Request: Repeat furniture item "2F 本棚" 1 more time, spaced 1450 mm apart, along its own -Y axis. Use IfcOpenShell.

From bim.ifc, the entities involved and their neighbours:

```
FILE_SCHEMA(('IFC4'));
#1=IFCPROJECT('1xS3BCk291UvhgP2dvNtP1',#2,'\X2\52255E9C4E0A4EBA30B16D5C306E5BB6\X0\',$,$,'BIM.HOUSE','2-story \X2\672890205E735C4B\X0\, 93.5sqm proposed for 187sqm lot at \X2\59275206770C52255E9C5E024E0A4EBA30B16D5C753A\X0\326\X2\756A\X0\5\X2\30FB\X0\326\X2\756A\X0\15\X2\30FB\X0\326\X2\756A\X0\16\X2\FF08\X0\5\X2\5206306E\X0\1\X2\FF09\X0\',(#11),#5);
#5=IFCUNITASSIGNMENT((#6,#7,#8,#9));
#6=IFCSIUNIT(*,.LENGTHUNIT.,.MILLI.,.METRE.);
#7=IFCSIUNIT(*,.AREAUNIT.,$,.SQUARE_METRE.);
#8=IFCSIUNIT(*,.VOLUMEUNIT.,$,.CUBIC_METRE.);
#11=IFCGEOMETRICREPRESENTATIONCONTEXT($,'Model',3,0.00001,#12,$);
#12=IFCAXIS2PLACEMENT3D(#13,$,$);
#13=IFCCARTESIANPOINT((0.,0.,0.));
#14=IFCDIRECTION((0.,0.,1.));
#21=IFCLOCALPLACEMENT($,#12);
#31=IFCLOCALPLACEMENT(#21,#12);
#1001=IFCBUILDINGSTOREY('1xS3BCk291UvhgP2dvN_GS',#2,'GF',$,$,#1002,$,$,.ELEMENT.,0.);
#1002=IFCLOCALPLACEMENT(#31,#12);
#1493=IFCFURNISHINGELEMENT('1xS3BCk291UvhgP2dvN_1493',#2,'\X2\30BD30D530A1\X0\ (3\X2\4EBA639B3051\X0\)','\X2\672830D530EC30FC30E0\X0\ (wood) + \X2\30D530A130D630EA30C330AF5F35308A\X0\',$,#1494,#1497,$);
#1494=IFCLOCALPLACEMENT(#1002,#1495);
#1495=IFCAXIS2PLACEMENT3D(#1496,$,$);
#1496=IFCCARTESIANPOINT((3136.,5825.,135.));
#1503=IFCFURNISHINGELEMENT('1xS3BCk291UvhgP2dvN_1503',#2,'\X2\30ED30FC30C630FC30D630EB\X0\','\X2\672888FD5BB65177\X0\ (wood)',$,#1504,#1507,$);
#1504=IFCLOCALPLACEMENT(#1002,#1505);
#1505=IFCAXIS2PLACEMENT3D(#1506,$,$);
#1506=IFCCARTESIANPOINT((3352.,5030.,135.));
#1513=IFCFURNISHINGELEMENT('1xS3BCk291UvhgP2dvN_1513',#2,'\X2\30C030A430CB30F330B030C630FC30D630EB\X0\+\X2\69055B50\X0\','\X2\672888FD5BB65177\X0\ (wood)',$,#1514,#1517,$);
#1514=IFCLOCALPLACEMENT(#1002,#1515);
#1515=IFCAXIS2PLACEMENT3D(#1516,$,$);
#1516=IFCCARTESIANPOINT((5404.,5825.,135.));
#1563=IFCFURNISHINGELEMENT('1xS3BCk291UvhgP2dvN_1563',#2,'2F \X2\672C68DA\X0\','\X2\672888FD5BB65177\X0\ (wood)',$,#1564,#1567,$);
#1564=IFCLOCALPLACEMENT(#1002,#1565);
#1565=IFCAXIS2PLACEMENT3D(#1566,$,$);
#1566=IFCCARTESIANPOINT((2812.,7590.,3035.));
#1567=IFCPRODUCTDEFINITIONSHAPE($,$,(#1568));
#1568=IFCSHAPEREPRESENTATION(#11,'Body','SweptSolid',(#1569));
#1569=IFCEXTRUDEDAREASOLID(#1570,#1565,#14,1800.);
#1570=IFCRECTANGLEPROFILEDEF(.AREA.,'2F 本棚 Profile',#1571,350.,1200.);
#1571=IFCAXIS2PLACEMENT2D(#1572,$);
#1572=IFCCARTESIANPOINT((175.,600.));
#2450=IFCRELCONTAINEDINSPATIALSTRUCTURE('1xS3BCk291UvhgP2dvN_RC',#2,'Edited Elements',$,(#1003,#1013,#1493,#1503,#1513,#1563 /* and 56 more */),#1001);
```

```python
import ifcopenshell
import ifcopenshell.api.geometry
import ifcopenshell.api.root
import ifcopenshell.util.element
import ifcopenshell.util.placement

model = ifcopenshell.open("bim.ifc")


def reuse_history(source, copy):
    """copy_class also copies each property set's owner history, people and application; keep the originals."""
    for rel in copy.IsDefinedBy:
        if rel.is_a("IfcRelDefinesByProperties") and (history := rel.RelatingPropertyDefinition.OwnerHistory):
            rel.RelatingPropertyDefinition.OwnerHistory = source.OwnerHistory
            ifcopenshell.util.element.remove_deep2(model, history)


source = model.by_guid("1xS3BCk291UvhgP2dvN_1563")
base = ifcopenshell.util.placement.get_local_placement(source.ObjectPlacement)
step = -base[:3, 1] * 1450.0

for i in range(1, 2):
    copy = ifcopenshell.api.root.copy_class(model, product=source)
    copy.Representation = ifcopenshell.util.element.copy_deep(
        model, source.Representation, exclude=["IfcGeometricRepresentationContext", "IfcRepresentationMap"]
    )
    reuse_history(source, copy)
    matrix = base.copy()
    matrix[:3, 3] += i * step
    print("added at", matrix[:3, 3].round(3) + 0.0)
    ifcopenshell.api.geometry.edit_object_placement(model, product=copy, matrix=matrix, is_si=False)

model.write("bim_updated.ifc")
```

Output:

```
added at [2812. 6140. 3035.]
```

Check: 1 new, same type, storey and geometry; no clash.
